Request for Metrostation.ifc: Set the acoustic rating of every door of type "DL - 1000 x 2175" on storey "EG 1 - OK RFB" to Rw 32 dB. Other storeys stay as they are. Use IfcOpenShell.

First a look at what the model holds.

```python
import ifcopenshell
import ifcopenshell.util.element

model = ifcopenshell.open("Metrostation.ifc")
print(model.schema)
storey = next(s for s in model.by_type("IfcBuildingStorey") if s.Name == "EG 1 - OK RFB")
doors = [e for e in ifcopenshell.util.element.get_decomposition(storey) if e.is_a("IfcDoor")]
seen = {}
for e in doors:
    element_type = ifcopenshell.util.element.get_type(e)
    key = (element_type.Name if element_type != e and element_type else None, ifcopenshell.util.element.get_pset(e, "Pset_DoorCommon", "AcousticRating"))
    seen[key] = seen.get(key, 0) + 1
for (name, value), count in sorted(seen.items(), key=str):
    print(count, "x", name, "|", value)
```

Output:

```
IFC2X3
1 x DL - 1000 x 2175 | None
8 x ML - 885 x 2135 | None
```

```python
import ifcopenshell
import ifcopenshell.api.pset
import ifcopenshell.util.element

model = ifcopenshell.open("Metrostation.ifc")

storey = next(s for s in model.by_type("IfcBuildingStorey") if s.Name == "EG 1 - OK RFB")
doors = [e for e in ifcopenshell.util.element.get_decomposition(storey) if e.is_a("IfcDoor")]

count = 0
for e in doors:
    element_type = ifcopenshell.util.element.get_type(e)
    if element_type in (None, e) or element_type.Name != "DL - 1000 x 2175":
        continue
    # add_pset returns the element's existing set when there is one.
    pset = ifcopenshell.api.pset.add_pset(model, product=e, name="Pset_DoorCommon")
    ifcopenshell.api.pset.edit_pset(model, pset=pset, properties={"AcousticRating": "Rw 32 dB"})
    count += 1

print(count, "doors updated")

model.write("Metrostation_edited.ifc")
```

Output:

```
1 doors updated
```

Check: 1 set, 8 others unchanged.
